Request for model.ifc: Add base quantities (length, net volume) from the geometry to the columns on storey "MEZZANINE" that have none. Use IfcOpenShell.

First a look at what the model holds.

```python
import ifcopenshell
import ifcopenshell.util.element
import ifcopenshell.util.unit

model = ifcopenshell.open("model.ifc")
print(model.schema)
for unit_type in ("LENGTHUNIT", "AREAUNIT", "VOLUMEUNIT"):
    print(unit_type, ifcopenshell.util.unit.calculate_unit_scale(model, unit_type))
storey = next(s for s in model.by_type("IfcBuildingStorey") if s.Name == "MEZZANINE")
columns = [e for e in ifcopenshell.util.element.get_decomposition(storey) if e.is_a("IfcColumn")]
for e in sorted(columns, key=lambda e: e.id()):
    print(e.id(), e.is_a(), e.Name, list(ifcopenshell.util.element.get_psets(e, qtos_only=True)), sep=" | ")
```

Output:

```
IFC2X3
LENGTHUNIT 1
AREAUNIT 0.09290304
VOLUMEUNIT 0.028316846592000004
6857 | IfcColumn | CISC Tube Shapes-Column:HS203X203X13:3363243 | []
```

```python
import ifcopenshell
import ifcopenshell.api.pset
import ifcopenshell.geom
import ifcopenshell.util.element
import ifcopenshell.util.shape
import ifcopenshell.util.unit

model = ifcopenshell.open("model.ifc")
unit_scale = ifcopenshell.util.unit.calculate_unit_scale(model)
volume_scale = ifcopenshell.util.unit.calculate_unit_scale(model, "VOLUMEUNIT")
settings = ifcopenshell.geom.settings()

storey = next(s for s in model.by_type("IfcBuildingStorey") if s.Name == "MEZZANINE")
columns = [e for e in ifcopenshell.util.element.get_decomposition(storey) if e.is_a("IfcColumn")]

for e in sorted(columns, key=lambda e: e.id()):
    if ifcopenshell.util.element.get_psets(e, qtos_only=True, should_inherit=False):
        continue
    # Geometry comes back in metres, in the element's own axes.
    shape = ifcopenshell.geom.create_shape(settings, e)
    values = {
        "Length": ifcopenshell.util.shape.get_z(shape.geometry) / unit_scale,
        "NetVolume": ifcopenshell.util.shape.get_volume(shape.geometry) / volume_scale,
    }
    qto = ifcopenshell.api.pset.add_qto(model, product=e, name="BaseQuantities")
    ifcopenshell.api.pset.edit_qto(model, qto=qto, properties=values)
    print(e.id(), {k: round(v, 3) for k, v in values.items()})

model.write("model_rev.ifc")
```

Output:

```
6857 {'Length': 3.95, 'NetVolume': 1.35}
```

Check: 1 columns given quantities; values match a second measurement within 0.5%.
